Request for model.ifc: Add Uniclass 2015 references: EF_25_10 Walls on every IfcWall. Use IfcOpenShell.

First a look at what the model holds.

```python
import ifcopenshell

model = ifcopenshell.open("model.ifc")
print(model.schema)
print("classifications:", [c.Name for c in model.by_type("IfcClassification")])
for ifc_class in ("IfcDoor", "IfcRoof", "IfcStair", "IfcWall", "IfcWindow"):
    print(ifc_class, len(model.by_type(ifc_class)))
```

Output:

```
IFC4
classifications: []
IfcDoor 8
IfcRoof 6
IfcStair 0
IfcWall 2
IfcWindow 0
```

```python
import ifcopenshell
import ifcopenshell.api.classification

model = ifcopenshell.open("model.ifc")

system = ifcopenshell.api.classification.add_classification(model, classification="Uniclass 2015")

codes = {
    "IfcWall": ("EF_25_10", "Walls"),
}
for ifc_class, (code, name) in codes.items():
    products = model.by_type(ifc_class)
    ifcopenshell.api.classification.add_reference(
        model, products=products, classification=system, identification=code, name=name
    )
    print(code, len(products))

model.write("model_rev.ifc")
```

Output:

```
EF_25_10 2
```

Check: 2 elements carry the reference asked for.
